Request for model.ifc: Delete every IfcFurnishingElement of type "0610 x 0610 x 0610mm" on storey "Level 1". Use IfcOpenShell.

First a look at what the model holds.

```python
import ifcopenshell
import ifcopenshell.util.element

model = ifcopenshell.open("model.ifc")
print(model.schema)
storey = next(s for s in model.by_type("IfcBuildingStorey") if s.Name == "Level 1")
furniture = [e for e in ifcopenshell.util.element.get_decomposition(storey) if e.is_a("IfcFurnishingElement")]
seen = {}
for e in furniture:
    element_type = ifcopenshell.util.element.get_type(e)
    name = element_type.Name if element_type not in (None, e) else None
    seen[name] = seen.get(name, 0) + 1
for name, count in sorted(seen.items(), key=str):
    print(count, "x", name)
```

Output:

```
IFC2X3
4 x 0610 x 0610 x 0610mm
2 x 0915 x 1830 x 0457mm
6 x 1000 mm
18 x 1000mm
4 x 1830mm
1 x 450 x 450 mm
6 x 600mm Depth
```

```python
import ifcopenshell
import ifcopenshell.api.root
import ifcopenshell.util.element

model = ifcopenshell.open("model.ifc")

storey = next(s for s in model.by_type("IfcBuildingStorey") if s.Name == "Level 1")
furniture = [e for e in ifcopenshell.util.element.get_decomposition(storey) if e.is_a("IfcFurnishingElement")]
targets = [e for e in furniture if (t := ifcopenshell.util.element.get_type(e)) not in (None, e) and t.Name == "0610 x 0610 x 0610mm"]

for e in targets:
    ifcopenshell.api.root.remove_product(model, product=e)
print(len(targets), "removed")

model.write("model_edited.ifc")
```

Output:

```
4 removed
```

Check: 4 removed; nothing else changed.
